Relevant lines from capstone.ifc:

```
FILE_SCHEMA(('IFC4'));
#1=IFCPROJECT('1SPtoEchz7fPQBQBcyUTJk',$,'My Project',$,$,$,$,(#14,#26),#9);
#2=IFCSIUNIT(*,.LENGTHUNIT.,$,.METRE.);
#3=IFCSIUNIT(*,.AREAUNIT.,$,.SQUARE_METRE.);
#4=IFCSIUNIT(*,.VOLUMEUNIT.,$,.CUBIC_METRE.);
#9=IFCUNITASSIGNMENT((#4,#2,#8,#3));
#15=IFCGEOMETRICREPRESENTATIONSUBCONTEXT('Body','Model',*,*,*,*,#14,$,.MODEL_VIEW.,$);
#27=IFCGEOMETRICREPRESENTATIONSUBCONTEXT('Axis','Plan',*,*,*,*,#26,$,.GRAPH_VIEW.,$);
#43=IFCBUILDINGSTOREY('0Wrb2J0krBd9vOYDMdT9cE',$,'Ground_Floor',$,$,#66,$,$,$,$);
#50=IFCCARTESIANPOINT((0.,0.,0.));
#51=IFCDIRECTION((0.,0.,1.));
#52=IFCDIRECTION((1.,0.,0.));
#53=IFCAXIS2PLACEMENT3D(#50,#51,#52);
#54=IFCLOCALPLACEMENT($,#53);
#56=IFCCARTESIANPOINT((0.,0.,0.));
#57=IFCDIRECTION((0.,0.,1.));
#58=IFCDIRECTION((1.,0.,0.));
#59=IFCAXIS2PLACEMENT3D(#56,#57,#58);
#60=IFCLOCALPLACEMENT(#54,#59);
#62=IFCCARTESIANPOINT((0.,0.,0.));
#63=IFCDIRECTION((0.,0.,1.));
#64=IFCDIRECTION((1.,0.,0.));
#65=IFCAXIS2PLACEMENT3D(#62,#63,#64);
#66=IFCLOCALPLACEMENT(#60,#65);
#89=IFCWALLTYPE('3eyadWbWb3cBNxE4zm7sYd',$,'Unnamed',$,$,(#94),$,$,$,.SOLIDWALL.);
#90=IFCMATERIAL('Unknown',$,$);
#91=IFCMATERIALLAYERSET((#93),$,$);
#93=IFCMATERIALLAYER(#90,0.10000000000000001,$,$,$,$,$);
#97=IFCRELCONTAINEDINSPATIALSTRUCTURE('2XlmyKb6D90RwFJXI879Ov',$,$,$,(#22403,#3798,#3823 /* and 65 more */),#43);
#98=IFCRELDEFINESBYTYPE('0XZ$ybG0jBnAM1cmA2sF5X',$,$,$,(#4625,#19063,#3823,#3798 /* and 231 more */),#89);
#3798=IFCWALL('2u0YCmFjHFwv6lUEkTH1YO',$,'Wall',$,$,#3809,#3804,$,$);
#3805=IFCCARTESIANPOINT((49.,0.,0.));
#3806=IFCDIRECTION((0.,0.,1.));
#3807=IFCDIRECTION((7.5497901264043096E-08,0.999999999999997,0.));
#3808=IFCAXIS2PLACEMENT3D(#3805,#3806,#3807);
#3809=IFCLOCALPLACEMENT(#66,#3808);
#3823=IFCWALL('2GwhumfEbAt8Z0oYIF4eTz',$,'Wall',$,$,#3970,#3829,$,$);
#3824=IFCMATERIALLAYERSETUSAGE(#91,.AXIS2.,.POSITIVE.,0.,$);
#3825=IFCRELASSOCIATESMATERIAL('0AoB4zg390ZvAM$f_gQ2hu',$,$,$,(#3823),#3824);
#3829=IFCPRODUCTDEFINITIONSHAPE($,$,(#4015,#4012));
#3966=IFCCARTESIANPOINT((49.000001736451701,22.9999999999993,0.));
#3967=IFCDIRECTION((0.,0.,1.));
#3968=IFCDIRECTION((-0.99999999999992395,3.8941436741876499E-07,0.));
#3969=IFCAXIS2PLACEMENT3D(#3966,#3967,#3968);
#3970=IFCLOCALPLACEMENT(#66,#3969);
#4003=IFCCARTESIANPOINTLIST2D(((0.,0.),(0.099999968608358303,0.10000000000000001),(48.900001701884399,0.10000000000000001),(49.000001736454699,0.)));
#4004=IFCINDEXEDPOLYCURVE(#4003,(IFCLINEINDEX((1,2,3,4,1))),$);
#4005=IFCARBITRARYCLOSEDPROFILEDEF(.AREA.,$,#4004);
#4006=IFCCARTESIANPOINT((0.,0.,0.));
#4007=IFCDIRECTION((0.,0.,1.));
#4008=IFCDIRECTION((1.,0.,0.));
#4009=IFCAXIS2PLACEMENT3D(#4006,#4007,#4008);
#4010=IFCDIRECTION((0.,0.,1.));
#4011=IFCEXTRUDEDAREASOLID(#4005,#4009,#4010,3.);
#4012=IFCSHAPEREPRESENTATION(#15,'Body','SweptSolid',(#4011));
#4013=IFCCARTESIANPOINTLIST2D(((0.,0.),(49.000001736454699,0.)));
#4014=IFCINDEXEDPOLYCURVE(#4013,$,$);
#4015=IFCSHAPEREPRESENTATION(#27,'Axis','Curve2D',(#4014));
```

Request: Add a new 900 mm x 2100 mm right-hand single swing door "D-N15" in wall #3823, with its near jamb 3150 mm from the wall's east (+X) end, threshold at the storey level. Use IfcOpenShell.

```python
import numpy as np
import ifcopenshell
import ifcopenshell.api.feature
import ifcopenshell.api.geometry
import ifcopenshell.api.root
import ifcopenshell.api.spatial
import ifcopenshell.geom
import ifcopenshell.util.element
import ifcopenshell.util.placement
import ifcopenshell.util.representation
import ifcopenshell.util.shape
import ifcopenshell.util.unit

model = ifcopenshell.open("capstone.ifc")
unit_scale = ifcopenshell.util.unit.calculate_unit_scale(model)
settings = ifcopenshell.geom.settings()


def volume(element):
    """Net volume in cubic metres, openings subtracted."""
    shape = ifcopenshell.geom.create_shape(settings, element)
    return ifcopenshell.util.shape.get_volume(shape.geometry)


wall = model.by_guid("2GwhumfEbAt8Z0oYIF4eTz")
storey = ifcopenshell.util.element.get_container(wall, ifc_class="IfcBuildingStorey")
context = ifcopenshell.util.representation.get_context(model, "Model", "Body", "MODEL_VIEW")
before = volume(wall)

width, height, from_end, sill = 0.9, 2.1, 3.15, 0.0  # metres

# The wall runs along its own X axis, and the end named is its -X end.
wall_shape = ifcopenshell.geom.create_shape(settings, wall)
x, y, z = ifcopenshell.util.shape.get_vertices(wall_shape.geometry).T
start = x.min() + from_end
face, thickness = float(y.min()), float(y.max() - y.min())
wall_matrix = ifcopenshell.util.placement.get_local_placement(wall.ObjectPlacement)
level = ifcopenshell.util.placement.get_local_placement(storey.ObjectPlacement)[2, 3]


def in_wall(x, y):
    """Placement at x, y metres in the wall's axes, at sill height."""
    matrix = wall_matrix.copy()
    matrix[:, 3] = wall_matrix @ np.array([x / unit_scale, y / unit_scale, 0.0, 1.0])
    matrix[2, 3] = level + sill / unit_scale
    return matrix


# Opening: a box that overshoots both wall faces by 50 mm.
opening = ifcopenshell.api.root.create_entity(model, ifc_class="IfcOpeningElement", predefined_type="OPENING")
box = ifcopenshell.api.geometry.add_wall_representation(
    model, context=context, length=width, height=height, thickness=thickness + 0.1
)
ifcopenshell.api.geometry.assign_representation(model, product=opening, representation=box)
ifcopenshell.api.geometry.edit_object_placement(model, product=opening, matrix=in_wall(start, face - 0.05), is_si=False)
ifcopenshell.api.feature.add_feature(model, feature=opening, element=wall)

door = ifcopenshell.api.root.create_entity(model, ifc_class="IfcDoor", name="D-N15", predefined_type="DOOR")
door.OverallWidth, door.OverallHeight = width / unit_scale, height / unit_scale
door.OperationType = "SINGLE_SWING_RIGHT"
body = ifcopenshell.api.geometry.add_door_representation(
    model,
    context=context,
    overall_width=door.OverallWidth,
    overall_height=door.OverallHeight,
    operation_type="SINGLE_SWING_RIGHT",
    lining_properties={"LiningDepth": thickness / unit_scale, "ThresholdDepth": thickness / unit_scale},
)
ifcopenshell.api.geometry.assign_representation(model, product=door, representation=body)
ifcopenshell.api.spatial.assign_container(model, products=[door], relating_structure=storey)
ifcopenshell.api.feature.add_filling(model, opening=opening, element=door)

# The lining spans the wall, so the door starts at the wall face.
ifcopenshell.api.geometry.edit_object_placement(model, product=door, matrix=in_wall(start, face), is_si=False)

after = volume(wall)

print(f"wall volume {before:.3f} -> {after:.3f} m3")

model.write("capstone_rev.ifc")
```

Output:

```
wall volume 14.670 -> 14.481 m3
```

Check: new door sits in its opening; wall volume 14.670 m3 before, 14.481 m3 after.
